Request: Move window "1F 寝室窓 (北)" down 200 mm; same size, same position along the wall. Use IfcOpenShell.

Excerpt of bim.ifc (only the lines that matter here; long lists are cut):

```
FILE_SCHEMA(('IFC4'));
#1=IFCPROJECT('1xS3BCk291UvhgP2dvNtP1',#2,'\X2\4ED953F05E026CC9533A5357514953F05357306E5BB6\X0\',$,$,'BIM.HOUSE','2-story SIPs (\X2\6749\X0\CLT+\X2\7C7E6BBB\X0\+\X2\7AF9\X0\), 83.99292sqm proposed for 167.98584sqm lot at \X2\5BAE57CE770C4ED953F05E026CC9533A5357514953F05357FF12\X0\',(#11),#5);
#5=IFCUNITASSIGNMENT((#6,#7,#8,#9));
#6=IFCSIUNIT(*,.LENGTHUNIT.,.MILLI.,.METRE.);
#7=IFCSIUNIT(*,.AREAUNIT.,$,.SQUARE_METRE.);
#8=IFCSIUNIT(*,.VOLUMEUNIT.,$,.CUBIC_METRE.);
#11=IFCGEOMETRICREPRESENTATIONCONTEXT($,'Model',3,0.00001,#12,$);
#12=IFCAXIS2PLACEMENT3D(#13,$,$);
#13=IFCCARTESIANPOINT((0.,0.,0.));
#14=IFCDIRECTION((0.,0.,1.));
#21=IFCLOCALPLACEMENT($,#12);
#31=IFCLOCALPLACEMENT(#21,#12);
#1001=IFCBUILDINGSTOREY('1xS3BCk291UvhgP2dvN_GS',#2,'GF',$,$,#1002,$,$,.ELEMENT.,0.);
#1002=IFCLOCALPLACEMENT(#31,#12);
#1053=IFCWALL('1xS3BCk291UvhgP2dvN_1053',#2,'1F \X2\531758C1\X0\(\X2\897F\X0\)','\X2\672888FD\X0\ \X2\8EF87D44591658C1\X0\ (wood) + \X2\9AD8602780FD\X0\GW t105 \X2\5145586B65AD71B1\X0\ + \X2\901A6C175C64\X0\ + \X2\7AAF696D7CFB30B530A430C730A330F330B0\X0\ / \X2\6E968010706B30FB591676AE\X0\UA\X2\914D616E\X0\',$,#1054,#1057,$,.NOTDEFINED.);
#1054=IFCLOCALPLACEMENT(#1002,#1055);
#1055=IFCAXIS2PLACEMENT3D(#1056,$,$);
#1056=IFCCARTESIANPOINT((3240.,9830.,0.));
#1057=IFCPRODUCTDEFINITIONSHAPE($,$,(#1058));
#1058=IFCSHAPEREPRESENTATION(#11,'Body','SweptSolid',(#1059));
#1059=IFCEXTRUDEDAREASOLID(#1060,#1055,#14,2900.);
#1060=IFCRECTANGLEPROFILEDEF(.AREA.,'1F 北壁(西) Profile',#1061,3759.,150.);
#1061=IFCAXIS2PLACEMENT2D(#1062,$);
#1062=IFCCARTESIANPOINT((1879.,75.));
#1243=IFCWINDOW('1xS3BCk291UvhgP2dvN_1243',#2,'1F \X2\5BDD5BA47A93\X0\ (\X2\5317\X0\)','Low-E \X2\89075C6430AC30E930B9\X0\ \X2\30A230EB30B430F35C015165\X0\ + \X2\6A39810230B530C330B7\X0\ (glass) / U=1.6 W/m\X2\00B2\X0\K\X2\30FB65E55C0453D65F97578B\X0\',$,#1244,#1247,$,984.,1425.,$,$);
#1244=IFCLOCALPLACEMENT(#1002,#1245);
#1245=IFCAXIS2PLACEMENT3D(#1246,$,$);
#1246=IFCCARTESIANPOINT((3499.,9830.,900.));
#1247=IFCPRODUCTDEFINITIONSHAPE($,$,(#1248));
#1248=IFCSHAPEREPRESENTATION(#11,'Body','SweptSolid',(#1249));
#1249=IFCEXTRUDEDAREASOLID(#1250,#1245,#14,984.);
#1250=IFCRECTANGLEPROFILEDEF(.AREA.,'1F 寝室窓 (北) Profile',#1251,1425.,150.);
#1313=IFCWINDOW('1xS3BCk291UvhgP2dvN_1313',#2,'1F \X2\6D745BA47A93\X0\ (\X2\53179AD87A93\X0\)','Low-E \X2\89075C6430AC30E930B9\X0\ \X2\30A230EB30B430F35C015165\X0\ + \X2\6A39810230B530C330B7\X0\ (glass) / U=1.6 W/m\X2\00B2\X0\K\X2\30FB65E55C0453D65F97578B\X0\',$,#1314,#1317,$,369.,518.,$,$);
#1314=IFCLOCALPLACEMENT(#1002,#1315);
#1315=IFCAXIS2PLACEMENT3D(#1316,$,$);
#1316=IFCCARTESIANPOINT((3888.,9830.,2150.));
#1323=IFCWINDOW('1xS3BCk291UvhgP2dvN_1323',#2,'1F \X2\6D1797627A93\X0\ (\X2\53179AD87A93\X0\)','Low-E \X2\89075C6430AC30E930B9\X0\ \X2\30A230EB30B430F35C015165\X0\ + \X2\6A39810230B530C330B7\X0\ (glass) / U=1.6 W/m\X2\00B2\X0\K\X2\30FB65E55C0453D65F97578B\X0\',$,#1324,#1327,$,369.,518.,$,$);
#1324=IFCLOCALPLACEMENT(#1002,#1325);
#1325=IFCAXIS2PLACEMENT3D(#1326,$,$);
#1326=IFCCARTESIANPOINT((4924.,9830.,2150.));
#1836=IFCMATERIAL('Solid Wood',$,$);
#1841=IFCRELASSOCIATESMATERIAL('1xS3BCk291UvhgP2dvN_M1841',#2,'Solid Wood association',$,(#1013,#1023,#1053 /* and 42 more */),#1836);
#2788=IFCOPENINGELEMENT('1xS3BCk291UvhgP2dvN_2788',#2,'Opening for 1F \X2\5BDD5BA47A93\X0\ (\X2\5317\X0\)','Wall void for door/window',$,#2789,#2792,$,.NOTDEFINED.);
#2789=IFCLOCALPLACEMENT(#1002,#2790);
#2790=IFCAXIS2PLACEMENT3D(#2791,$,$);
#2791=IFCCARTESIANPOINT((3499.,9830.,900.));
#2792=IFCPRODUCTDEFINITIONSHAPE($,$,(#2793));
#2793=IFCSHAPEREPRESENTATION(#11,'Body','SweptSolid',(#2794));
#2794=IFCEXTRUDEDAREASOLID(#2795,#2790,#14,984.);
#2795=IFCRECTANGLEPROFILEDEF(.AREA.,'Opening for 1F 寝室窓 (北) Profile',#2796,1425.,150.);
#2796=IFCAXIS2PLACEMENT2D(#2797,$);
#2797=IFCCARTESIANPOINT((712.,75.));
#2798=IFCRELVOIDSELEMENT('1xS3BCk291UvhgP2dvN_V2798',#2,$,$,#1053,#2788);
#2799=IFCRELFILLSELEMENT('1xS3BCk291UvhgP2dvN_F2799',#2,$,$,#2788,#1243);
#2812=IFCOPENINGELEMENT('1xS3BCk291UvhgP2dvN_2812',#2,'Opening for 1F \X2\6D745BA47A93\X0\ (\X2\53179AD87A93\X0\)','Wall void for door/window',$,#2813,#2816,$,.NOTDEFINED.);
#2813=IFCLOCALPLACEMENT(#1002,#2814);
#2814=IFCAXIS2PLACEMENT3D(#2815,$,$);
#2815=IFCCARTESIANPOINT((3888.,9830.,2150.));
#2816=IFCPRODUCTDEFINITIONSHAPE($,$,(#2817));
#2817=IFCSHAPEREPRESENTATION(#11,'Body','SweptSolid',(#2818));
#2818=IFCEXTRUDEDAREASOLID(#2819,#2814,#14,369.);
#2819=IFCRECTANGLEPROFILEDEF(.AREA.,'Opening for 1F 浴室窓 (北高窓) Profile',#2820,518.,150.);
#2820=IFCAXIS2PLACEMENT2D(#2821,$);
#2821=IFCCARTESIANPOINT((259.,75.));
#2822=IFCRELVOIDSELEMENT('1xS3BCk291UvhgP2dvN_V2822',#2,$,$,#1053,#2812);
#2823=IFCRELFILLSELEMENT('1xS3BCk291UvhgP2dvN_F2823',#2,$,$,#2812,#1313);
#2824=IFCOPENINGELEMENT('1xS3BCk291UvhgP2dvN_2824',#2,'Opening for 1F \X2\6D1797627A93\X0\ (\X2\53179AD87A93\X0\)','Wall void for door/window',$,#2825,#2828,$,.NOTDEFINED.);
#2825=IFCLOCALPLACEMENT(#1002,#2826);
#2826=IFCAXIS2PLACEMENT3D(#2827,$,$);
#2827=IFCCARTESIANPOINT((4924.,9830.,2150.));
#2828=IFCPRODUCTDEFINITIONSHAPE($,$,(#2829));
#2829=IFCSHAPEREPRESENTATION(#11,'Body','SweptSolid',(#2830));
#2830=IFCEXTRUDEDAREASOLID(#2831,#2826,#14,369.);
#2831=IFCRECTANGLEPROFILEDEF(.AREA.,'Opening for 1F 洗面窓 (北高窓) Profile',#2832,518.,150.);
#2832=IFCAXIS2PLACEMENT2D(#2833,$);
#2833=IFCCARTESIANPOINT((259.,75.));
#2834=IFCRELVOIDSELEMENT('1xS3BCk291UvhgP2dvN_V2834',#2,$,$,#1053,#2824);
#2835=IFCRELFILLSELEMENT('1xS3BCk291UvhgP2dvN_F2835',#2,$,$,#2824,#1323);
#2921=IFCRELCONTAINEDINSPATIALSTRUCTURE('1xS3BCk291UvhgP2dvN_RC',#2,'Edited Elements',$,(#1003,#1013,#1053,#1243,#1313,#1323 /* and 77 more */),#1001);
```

```python
import numpy as np
import ifcopenshell
import ifcopenshell.api.geometry
import ifcopenshell.util.placement
import ifcopenshell.util.unit

model = ifcopenshell.open("bim.ifc")
unit_scale = ifcopenshell.util.unit.calculate_unit_scale(model)

window = model.by_id(1243)
opening = window.FillsVoids[0].RelatingOpeningElement
dz = -0.2 / unit_scale

shift = np.array([0.0, 0.0, dz])
# The window is not placed relative to its opening, so move both.
for product in (opening, window):
    matrix = ifcopenshell.util.placement.get_local_placement(product.ObjectPlacement)
    matrix[:3, 3] += shift
    ifcopenshell.api.geometry.edit_object_placement(model, product=product, matrix=matrix, is_si=False)

print(f"moved by {dz * unit_scale:+.3f} m")

model.write("bim_updated.ifc")
```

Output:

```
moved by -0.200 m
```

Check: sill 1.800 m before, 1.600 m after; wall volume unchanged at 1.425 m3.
